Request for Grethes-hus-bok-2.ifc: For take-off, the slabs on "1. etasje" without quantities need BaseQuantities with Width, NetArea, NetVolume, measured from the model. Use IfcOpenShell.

First a look at what the model holds.

```python
import ifcopenshell
import ifcopenshell.util.element
import ifcopenshell.util.unit

model = ifcopenshell.open("Grethes-hus-bok-2.ifc")
print(model.schema)
for unit_type in ("LENGTHUNIT", "AREAUNIT", "VOLUMEUNIT"):
    print(unit_type, ifcopenshell.util.unit.calculate_unit_scale(model, unit_type))
storey = next(s for s in model.by_type("IfcBuildingStorey") if s.Name == "1. etasje")
slabs = [e for e in ifcopenshell.util.element.get_decomposition(storey) if e.is_a("IfcSlab")]
for e in sorted(slabs, key=lambda e: e.id()):
    print(e.id(), e.is_a(), e.Name, list(ifcopenshell.util.element.get_psets(e, qtos_only=True)), sep=" | ")
```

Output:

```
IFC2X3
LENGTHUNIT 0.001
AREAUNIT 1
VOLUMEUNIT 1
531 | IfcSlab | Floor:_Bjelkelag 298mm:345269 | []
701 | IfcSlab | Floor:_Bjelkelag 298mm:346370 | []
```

```python
import ifcopenshell
import ifcopenshell.api.pset
import ifcopenshell.geom
import ifcopenshell.util.element
import ifcopenshell.util.shape
import ifcopenshell.util.unit

model = ifcopenshell.open("Grethes-hus-bok-2.ifc")
unit_scale = ifcopenshell.util.unit.calculate_unit_scale(model)
area_scale = ifcopenshell.util.unit.calculate_unit_scale(model, "AREAUNIT")
volume_scale = ifcopenshell.util.unit.calculate_unit_scale(model, "VOLUMEUNIT")
settings = ifcopenshell.geom.settings()

storey = next(s for s in model.by_type("IfcBuildingStorey") if s.Name == "1. etasje")
slabs = [e for e in ifcopenshell.util.element.get_decomposition(storey) if e.is_a("IfcSlab")]

for e in sorted(slabs, key=lambda e: e.id()):
    if ifcopenshell.util.element.get_psets(e, qtos_only=True, should_inherit=False):
        continue
    # Geometry comes back in metres, in the element's own axes.
    shape = ifcopenshell.geom.create_shape(settings, e)
    values = {
        "Width": ifcopenshell.util.shape.get_z(shape.geometry) / unit_scale,
        "NetArea": ifcopenshell.util.shape.get_footprint_area(shape.geometry) / area_scale,
        "NetVolume": ifcopenshell.util.shape.get_volume(shape.geometry) / volume_scale,
    }
    qto = ifcopenshell.api.pset.add_qto(model, product=e, name="BaseQuantities")
    ifcopenshell.api.pset.edit_qto(model, qto=qto, properties=values)
    print(e.id(), {k: round(v, 3) for k, v in values.items()})

model.write("Grethes-hus-bok-2_rev.ifc")
```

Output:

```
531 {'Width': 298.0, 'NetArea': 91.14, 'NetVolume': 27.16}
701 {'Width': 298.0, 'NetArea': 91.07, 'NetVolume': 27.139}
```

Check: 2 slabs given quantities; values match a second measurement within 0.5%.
